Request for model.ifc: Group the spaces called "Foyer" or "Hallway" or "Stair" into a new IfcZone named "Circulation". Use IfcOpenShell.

First a look at what the model holds.

```python
import ifcopenshell

model = ifcopenshell.open("model.ifc")
print(model.schema)
seen = {}
for space in model.by_type("IfcSpace"):
    seen[space.LongName] = seen.get(space.LongName, 0) + 1
for name, count in sorted(seen.items(), key=str):
    print(count, "x", name)
print("zones:", [z.Name for z in model.by_type("IfcZone")][:20])
```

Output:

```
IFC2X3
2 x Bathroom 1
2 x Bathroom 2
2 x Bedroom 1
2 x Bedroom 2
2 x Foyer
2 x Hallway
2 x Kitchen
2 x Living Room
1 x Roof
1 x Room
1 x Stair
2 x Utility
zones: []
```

```python
import ifcopenshell
import ifcopenshell.api.group
import ifcopenshell.api.root

model = ifcopenshell.open("model.ifc")

names = {"Foyer", "Hallway", "Stair"}
spaces = [s for s in model.by_type("IfcSpace") if s.LongName in names]

zone = ifcopenshell.api.root.create_entity(model, ifc_class="IfcZone", name="Circulation")
ifcopenshell.api.group.assign_group(model, products=spaces, group=zone)
print(len(spaces), "spaces in", zone.Name)

model.write("model_rev.ifc")
```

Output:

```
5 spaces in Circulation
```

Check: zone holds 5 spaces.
